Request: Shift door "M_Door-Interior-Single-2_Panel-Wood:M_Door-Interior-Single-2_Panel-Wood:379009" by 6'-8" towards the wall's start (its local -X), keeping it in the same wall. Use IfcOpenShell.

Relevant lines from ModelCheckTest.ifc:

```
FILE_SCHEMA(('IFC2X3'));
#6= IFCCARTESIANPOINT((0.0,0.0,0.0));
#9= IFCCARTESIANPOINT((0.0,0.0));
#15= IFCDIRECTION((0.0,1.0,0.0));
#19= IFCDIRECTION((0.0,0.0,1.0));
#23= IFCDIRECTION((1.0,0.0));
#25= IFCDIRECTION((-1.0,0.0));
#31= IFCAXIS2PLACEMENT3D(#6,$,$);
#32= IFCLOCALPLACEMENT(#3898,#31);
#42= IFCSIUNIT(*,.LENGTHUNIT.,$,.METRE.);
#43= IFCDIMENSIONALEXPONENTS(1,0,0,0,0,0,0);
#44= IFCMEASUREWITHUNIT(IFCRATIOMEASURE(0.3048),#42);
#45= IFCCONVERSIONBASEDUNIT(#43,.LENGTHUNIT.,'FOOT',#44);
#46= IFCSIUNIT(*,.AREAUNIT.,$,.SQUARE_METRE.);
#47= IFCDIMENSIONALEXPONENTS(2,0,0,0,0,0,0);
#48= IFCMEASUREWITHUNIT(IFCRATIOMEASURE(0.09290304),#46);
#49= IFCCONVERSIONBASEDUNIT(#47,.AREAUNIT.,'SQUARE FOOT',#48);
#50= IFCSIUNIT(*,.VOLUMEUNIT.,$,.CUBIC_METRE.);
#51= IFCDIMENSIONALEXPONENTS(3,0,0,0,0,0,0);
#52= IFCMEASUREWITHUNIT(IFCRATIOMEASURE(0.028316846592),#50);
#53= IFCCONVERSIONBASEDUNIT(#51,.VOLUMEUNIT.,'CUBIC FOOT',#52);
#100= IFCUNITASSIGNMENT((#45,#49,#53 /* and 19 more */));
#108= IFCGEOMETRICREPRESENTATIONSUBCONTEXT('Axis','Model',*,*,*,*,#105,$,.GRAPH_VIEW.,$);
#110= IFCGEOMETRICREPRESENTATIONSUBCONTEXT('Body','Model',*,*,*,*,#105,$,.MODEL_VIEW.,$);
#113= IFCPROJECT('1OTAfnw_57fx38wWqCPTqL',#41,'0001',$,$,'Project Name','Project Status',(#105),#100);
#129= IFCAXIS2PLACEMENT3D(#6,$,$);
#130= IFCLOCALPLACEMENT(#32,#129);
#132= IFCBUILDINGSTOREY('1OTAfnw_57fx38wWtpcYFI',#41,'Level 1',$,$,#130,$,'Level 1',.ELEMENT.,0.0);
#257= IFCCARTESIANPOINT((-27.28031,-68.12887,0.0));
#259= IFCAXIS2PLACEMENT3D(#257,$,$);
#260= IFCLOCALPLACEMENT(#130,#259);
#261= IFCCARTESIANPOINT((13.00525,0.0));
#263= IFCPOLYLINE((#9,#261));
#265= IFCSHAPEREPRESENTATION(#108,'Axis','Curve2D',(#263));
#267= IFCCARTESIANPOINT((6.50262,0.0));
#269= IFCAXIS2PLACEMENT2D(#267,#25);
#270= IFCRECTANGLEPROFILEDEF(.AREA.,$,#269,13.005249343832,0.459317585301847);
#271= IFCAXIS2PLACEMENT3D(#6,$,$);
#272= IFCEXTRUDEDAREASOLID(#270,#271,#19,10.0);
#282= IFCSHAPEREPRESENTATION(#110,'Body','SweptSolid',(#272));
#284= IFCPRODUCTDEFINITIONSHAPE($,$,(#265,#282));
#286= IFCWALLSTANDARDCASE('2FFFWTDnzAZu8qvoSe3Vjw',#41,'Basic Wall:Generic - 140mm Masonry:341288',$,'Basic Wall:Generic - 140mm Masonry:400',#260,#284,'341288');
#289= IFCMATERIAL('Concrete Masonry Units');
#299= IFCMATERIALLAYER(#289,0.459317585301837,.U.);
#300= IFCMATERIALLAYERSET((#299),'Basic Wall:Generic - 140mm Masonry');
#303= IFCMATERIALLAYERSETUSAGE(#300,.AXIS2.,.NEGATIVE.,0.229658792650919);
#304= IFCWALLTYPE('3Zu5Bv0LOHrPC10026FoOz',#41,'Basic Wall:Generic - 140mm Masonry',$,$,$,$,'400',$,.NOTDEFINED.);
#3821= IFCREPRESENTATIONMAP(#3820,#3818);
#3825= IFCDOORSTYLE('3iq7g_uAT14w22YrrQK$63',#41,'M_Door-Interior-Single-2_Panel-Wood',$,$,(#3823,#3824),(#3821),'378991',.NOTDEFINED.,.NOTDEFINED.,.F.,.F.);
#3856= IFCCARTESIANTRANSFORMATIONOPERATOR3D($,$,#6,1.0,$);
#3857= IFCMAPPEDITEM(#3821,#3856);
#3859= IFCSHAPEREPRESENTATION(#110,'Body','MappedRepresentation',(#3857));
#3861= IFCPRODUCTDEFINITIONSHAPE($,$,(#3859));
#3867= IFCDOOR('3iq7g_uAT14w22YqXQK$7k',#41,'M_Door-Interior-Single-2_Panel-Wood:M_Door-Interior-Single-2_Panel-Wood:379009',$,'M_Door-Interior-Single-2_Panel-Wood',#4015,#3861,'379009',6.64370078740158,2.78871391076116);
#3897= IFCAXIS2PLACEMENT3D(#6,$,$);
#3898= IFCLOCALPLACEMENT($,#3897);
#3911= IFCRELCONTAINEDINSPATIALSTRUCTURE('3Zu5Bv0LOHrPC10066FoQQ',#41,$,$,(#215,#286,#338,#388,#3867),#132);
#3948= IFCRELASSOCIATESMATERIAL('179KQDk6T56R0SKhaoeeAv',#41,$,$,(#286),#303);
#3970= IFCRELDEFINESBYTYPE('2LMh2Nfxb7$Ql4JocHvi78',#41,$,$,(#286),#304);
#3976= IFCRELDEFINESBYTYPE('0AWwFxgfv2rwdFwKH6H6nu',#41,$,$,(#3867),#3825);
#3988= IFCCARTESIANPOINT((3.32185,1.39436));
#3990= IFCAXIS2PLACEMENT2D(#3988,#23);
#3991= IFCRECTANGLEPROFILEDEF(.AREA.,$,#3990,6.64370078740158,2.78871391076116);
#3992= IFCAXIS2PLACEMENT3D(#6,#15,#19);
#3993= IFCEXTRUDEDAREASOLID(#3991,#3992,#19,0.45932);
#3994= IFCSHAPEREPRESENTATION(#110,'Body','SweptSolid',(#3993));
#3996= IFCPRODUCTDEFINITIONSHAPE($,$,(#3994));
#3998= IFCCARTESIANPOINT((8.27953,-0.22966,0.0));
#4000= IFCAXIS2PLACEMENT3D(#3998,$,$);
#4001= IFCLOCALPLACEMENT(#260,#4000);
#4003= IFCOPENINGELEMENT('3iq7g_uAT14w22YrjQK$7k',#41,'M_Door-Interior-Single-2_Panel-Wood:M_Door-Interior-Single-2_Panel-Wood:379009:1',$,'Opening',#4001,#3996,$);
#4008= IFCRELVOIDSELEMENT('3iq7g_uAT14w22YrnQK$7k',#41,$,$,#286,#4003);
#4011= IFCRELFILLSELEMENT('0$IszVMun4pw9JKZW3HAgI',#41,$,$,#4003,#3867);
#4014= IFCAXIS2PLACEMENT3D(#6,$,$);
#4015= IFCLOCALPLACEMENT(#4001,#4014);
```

```python
import ifcopenshell
import ifcopenshell.api.geometry
import ifcopenshell.util.placement
import ifcopenshell.util.unit

model = ifcopenshell.open("ModelCheckTest.ifc")
unit_scale = ifcopenshell.util.unit.calculate_unit_scale(model)

door = model.by_id(3867)
opening = door.FillsVoids[0].RelatingOpeningElement
wall = opening.VoidsElements[0].RelatingBuildingElement

wall_matrix = ifcopenshell.util.placement.get_local_placement(wall.ObjectPlacement)
shift = wall_matrix[:3, 0] * -80 * 0.0254 / unit_scale
before = ifcopenshell.util.placement.get_local_placement(door.ObjectPlacement)[:3, 3].copy()

# The door is placed relative to its opening, so it follows when the opening moves.
matrix = ifcopenshell.util.placement.get_local_placement(opening.ObjectPlacement)
matrix[:3, 3] += shift
ifcopenshell.api.geometry.edit_object_placement(
    model, product=opening, matrix=matrix, is_si=False, should_transform_children=True
)

after = ifcopenshell.util.placement.get_local_placement(door.ObjectPlacement)[:3, 3]
print("door moved by", (after - before).round(3) + 0.0)

model.write("ModelCheckTest_updated.ifc")
```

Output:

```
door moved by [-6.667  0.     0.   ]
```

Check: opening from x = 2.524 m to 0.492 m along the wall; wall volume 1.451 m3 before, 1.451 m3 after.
